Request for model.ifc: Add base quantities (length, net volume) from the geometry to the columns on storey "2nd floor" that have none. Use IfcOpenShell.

First a look at what the model holds.

```python
import ifcopenshell
import ifcopenshell.util.element
import ifcopenshell.util.unit

model = ifcopenshell.open("model.ifc")
print(model.schema)
for unit_type in ("LENGTHUNIT", "AREAUNIT", "VOLUMEUNIT"):
    print(unit_type, ifcopenshell.util.unit.calculate_unit_scale(model, unit_type))
storey = next(s for s in model.by_type("IfcBuildingStorey") if s.Name == "2nd floor")
columns = [e for e in ifcopenshell.util.element.get_decomposition(storey) if e.is_a("IfcColumn")]
for e in sorted(columns, key=lambda e: e.id()):
    print(e.id(), e.is_a(), e.Name, list(ifcopenshell.util.element.get_psets(e, qtos_only=True)), sep=" | ")
```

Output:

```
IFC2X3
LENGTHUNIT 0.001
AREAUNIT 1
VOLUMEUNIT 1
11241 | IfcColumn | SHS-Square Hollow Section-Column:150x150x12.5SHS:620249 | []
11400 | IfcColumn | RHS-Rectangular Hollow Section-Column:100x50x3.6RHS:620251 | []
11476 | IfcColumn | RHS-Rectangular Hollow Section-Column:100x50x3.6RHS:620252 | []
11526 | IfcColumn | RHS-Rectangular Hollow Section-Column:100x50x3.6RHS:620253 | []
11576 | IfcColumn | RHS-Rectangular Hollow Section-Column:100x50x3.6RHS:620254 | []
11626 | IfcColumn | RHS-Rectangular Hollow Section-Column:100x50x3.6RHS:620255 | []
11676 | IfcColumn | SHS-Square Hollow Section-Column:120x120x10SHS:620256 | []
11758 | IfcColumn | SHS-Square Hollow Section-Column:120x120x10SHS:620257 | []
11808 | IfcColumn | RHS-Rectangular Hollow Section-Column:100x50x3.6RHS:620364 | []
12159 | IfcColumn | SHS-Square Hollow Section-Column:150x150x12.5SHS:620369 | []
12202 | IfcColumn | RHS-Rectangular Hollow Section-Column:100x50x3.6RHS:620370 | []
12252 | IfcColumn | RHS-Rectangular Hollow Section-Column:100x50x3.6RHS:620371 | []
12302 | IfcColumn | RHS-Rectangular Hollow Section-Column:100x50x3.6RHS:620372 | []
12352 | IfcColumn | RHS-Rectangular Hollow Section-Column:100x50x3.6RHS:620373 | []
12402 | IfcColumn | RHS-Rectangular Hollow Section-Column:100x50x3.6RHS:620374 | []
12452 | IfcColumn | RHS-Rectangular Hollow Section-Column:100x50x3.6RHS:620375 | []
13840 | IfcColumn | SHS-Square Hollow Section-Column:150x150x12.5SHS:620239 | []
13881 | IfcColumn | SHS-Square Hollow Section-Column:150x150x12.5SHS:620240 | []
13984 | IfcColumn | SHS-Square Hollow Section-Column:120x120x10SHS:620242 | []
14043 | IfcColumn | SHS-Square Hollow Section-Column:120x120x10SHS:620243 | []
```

```python
import ifcopenshell
import ifcopenshell.api.pset
import ifcopenshell.geom
import ifcopenshell.util.element
import ifcopenshell.util.shape
import ifcopenshell.util.unit

model = ifcopenshell.open("model.ifc")
unit_scale = ifcopenshell.util.unit.calculate_unit_scale(model)
volume_scale = ifcopenshell.util.unit.calculate_unit_scale(model, "VOLUMEUNIT")
settings = ifcopenshell.geom.settings()

storey = next(s for s in model.by_type("IfcBuildingStorey") if s.Name == "2nd floor")
columns = [e for e in ifcopenshell.util.element.get_decomposition(storey) if e.is_a("IfcColumn")]

for e in sorted(columns, key=lambda e: e.id()):
    if ifcopenshell.util.element.get_psets(e, qtos_only=True, should_inherit=False):
        continue
    # Geometry comes back in metres, in the element's own axes.
    shape = ifcopenshell.geom.create_shape(settings, e)
    values = {
        "Length": ifcopenshell.util.shape.get_z(shape.geometry) / unit_scale,
        "NetVolume": ifcopenshell.util.shape.get_volume(shape.geometry) / volume_scale,
    }
    qto = ifcopenshell.api.pset.add_qto(model, product=e, name="BaseQuantities")
    ifcopenshell.api.pset.edit_qto(model, qto=qto, properties=values)
    print(e.id(), {k: round(v, 3) for k, v in values.items()})

model.write("model_rev.ifc")
```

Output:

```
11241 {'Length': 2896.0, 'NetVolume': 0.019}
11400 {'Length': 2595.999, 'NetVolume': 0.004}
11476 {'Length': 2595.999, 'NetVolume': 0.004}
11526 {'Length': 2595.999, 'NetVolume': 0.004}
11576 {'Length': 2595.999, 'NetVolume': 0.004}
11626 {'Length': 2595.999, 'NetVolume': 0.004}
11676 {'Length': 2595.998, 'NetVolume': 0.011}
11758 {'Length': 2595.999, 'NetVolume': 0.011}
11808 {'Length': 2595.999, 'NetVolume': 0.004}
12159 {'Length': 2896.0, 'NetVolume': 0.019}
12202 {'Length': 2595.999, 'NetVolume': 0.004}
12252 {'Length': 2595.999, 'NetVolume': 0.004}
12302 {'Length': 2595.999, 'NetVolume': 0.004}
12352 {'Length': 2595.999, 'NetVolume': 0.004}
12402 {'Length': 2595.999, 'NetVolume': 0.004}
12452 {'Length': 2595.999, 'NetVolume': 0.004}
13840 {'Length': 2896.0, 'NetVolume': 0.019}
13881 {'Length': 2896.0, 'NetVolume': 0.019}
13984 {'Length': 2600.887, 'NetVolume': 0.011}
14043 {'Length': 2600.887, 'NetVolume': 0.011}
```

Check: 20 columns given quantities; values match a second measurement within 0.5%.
